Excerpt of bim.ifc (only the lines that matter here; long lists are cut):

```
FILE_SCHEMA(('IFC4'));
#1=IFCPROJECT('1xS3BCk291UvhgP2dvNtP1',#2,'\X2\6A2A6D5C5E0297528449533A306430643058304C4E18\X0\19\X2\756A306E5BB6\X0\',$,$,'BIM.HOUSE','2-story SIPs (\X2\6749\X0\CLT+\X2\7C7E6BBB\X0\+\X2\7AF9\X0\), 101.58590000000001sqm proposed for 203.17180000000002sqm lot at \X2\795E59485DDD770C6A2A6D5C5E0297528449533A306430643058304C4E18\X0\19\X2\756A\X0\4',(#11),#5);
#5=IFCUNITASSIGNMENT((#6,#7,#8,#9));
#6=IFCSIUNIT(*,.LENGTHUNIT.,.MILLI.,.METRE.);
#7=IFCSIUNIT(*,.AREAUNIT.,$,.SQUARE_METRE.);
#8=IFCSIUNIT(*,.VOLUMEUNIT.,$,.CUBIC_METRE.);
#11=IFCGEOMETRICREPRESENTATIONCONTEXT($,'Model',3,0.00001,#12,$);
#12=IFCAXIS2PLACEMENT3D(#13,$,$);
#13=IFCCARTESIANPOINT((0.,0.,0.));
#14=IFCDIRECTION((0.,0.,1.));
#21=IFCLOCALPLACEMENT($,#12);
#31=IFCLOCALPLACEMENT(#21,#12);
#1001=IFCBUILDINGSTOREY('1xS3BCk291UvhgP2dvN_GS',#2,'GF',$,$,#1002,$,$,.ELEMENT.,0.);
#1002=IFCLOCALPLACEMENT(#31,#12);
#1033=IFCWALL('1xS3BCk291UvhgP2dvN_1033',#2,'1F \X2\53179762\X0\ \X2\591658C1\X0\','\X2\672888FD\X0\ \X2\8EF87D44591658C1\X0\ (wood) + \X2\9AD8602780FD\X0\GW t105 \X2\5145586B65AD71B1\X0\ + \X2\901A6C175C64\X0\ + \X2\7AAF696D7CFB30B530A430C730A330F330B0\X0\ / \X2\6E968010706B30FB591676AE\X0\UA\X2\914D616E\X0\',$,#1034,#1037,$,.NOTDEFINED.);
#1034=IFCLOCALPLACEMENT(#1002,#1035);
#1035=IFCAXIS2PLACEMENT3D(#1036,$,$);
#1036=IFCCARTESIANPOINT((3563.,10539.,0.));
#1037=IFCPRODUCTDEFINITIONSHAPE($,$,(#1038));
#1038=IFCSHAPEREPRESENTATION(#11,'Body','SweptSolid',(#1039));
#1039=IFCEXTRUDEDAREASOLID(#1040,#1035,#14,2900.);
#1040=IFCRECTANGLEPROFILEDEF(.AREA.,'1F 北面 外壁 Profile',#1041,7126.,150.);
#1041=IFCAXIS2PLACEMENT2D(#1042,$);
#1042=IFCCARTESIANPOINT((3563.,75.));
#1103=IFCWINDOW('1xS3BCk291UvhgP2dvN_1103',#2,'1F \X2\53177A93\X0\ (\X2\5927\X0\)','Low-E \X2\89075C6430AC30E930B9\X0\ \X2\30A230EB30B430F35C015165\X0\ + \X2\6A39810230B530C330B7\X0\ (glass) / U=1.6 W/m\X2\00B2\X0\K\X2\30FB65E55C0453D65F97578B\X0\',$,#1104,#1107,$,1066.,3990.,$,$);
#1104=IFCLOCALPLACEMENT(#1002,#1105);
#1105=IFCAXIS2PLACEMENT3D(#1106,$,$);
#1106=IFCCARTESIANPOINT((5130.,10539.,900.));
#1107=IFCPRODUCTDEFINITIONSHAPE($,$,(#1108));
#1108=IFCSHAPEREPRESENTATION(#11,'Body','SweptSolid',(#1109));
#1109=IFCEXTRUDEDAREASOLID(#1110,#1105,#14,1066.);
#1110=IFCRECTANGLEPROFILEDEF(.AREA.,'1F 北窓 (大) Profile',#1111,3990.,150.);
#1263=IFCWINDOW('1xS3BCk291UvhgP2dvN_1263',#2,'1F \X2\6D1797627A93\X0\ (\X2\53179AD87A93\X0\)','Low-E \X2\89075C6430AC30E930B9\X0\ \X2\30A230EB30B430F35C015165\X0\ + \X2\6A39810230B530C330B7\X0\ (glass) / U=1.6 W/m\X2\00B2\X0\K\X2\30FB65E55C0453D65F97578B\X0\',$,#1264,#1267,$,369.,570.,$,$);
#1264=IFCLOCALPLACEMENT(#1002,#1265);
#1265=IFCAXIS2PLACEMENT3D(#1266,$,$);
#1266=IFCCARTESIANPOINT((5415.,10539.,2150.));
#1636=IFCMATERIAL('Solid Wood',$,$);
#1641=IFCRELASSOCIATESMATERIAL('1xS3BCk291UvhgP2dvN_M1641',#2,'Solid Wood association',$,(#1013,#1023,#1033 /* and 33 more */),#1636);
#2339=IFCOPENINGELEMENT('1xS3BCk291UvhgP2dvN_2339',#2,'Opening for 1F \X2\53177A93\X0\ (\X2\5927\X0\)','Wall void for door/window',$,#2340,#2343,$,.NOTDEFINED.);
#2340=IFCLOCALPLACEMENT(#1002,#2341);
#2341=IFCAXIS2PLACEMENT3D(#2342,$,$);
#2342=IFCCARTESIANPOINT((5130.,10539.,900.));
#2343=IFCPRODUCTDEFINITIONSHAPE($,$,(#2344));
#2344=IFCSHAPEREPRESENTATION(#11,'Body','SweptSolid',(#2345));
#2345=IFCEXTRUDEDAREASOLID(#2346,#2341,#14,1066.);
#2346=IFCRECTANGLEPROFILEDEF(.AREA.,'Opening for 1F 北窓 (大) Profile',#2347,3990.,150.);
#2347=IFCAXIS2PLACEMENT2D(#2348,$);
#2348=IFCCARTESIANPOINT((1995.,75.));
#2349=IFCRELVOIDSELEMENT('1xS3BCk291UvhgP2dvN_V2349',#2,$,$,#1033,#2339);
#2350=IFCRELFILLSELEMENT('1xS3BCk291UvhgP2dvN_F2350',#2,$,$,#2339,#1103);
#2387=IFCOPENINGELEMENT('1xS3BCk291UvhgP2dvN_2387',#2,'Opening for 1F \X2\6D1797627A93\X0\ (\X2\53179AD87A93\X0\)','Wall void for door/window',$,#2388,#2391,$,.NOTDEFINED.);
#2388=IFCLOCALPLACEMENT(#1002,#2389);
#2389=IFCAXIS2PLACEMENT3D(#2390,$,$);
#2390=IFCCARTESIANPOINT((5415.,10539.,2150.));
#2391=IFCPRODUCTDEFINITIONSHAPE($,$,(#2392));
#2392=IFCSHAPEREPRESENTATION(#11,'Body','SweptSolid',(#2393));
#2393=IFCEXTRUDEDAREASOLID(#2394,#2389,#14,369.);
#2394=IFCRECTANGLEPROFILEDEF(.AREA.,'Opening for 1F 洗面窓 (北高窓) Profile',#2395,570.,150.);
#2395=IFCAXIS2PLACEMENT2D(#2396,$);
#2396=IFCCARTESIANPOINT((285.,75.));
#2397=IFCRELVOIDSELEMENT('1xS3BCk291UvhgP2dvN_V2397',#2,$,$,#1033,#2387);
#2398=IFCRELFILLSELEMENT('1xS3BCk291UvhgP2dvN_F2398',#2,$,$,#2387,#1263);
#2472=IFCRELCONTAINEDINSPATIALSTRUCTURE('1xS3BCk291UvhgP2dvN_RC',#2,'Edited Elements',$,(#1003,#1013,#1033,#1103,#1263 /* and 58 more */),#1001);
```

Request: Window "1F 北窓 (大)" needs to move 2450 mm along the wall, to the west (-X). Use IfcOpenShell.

```python
import ifcopenshell
import ifcopenshell.api.geometry
import ifcopenshell.util.placement

model = ifcopenshell.open("bim.ifc")

window = model.by_id(1103)
opening = window.FillsVoids[0].RelatingOpeningElement
wall = opening.VoidsElements[0].RelatingBuildingElement

wall_matrix = ifcopenshell.util.placement.get_local_placement(wall.ObjectPlacement)
shift = wall_matrix[:3, 0] * -2450.0
before = ifcopenshell.util.placement.get_local_placement(window.ObjectPlacement)[:3, 3].copy()

# The window is not placed relative to its opening, so move both.
for product in (opening, window):
    matrix = ifcopenshell.util.placement.get_local_placement(product.ObjectPlacement)
    matrix[:3, 3] += shift
    ifcopenshell.api.geometry.edit_object_placement(model, product=product, matrix=matrix, is_si=False)

after = ifcopenshell.util.placement.get_local_placement(window.ObjectPlacement)[:3, 3]
print("window moved by", (after - before).round(3) + 0.0)

model.write("bim_v2.ifc")
```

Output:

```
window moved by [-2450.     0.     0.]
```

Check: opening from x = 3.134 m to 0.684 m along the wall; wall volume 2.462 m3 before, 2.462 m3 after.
